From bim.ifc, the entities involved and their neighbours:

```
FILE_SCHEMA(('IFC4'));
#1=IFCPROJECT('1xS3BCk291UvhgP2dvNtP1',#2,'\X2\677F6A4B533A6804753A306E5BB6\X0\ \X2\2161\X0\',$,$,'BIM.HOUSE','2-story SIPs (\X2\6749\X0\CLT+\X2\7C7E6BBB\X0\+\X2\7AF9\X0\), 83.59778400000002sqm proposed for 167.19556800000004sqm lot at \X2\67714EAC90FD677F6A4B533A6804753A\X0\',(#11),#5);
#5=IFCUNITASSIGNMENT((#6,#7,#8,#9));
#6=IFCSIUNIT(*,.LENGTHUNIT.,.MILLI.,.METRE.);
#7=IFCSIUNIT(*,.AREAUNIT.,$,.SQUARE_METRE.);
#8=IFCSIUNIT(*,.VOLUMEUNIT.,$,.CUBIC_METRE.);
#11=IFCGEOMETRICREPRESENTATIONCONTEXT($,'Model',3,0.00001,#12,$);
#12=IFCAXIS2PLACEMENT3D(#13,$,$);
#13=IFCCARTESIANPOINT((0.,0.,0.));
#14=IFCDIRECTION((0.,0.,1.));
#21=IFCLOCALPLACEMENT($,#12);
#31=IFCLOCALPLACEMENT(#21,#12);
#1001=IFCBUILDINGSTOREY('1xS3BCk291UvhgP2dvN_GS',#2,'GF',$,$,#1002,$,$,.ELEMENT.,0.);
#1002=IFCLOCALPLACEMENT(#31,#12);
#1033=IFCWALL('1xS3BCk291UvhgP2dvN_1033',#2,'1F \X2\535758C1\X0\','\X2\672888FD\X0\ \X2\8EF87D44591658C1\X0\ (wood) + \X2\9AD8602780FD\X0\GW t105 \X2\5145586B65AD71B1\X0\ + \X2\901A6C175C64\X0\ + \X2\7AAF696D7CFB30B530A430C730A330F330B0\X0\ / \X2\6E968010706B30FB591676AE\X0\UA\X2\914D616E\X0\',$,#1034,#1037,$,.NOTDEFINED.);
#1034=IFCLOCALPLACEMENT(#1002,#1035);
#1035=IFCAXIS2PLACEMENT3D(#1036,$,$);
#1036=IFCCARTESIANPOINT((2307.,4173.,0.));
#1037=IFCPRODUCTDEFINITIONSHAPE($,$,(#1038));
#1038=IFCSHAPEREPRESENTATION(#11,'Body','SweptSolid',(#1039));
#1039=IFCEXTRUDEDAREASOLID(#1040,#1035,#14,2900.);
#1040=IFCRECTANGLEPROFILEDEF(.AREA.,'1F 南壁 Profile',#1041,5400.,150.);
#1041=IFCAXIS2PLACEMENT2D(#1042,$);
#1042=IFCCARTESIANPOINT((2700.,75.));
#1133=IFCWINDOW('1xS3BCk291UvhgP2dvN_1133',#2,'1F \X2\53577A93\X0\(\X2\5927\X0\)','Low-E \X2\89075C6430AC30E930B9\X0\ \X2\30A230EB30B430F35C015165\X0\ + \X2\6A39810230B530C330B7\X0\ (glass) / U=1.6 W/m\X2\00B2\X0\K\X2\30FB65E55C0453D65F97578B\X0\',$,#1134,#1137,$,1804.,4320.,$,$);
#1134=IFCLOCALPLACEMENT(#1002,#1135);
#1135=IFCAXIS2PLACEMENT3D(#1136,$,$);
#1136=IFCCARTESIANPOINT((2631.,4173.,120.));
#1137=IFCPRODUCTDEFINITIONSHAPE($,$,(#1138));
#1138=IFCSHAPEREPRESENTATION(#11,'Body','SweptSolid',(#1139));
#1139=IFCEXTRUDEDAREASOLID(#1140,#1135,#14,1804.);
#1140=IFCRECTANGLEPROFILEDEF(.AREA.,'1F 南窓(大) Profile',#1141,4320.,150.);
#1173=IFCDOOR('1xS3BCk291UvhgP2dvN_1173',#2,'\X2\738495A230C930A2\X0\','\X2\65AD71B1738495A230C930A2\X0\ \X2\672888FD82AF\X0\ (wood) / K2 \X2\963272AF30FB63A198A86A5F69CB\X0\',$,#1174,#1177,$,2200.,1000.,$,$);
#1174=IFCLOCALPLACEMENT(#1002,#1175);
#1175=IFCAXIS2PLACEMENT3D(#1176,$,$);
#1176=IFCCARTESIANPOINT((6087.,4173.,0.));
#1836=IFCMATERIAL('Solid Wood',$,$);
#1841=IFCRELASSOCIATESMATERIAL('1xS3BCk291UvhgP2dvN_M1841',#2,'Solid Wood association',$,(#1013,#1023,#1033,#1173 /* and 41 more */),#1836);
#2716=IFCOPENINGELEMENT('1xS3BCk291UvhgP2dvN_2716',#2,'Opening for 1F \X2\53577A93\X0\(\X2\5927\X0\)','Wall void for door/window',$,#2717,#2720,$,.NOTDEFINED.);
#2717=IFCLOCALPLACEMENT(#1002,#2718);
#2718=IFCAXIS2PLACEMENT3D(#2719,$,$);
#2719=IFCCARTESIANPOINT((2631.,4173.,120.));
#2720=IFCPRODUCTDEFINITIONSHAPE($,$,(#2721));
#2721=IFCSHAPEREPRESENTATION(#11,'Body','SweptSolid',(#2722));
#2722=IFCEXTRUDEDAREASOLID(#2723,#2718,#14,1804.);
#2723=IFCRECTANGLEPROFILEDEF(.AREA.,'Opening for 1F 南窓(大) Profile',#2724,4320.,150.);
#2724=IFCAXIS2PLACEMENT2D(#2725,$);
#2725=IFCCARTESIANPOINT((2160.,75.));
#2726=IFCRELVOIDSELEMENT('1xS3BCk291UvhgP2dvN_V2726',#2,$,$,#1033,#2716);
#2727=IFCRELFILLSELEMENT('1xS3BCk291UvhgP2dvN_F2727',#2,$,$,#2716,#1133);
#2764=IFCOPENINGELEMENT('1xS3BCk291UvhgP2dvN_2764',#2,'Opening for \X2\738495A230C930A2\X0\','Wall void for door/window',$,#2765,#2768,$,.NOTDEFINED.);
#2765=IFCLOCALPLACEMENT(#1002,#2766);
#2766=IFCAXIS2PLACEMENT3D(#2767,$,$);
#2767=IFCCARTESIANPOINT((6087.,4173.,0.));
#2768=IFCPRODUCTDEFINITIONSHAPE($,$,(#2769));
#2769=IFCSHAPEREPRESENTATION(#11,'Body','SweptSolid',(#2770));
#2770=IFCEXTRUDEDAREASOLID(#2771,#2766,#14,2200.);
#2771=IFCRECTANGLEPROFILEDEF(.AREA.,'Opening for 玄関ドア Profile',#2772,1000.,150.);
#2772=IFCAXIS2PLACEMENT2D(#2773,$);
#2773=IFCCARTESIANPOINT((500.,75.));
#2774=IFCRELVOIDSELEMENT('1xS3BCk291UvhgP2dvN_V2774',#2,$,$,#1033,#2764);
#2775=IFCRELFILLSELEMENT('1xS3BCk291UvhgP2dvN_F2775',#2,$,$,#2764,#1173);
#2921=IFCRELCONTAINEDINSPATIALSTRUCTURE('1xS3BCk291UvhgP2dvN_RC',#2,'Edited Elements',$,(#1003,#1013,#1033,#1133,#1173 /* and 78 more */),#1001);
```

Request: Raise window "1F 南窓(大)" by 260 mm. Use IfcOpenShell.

```python
import numpy as np
import ifcopenshell
import ifcopenshell.api.geometry
import ifcopenshell.util.placement
import ifcopenshell.util.unit

model = ifcopenshell.open("bim.ifc")
unit_scale = ifcopenshell.util.unit.calculate_unit_scale(model)

window = model.by_guid("1xS3BCk291UvhgP2dvN_1133")
opening = window.FillsVoids[0].RelatingOpeningElement
dz = 0.26 / unit_scale

shift = np.array([0.0, 0.0, dz])
# The window is not placed relative to its opening, so move both.
for product in (opening, window):
    matrix = ifcopenshell.util.placement.get_local_placement(product.ObjectPlacement)
    matrix[:3, 3] += shift
    ifcopenshell.api.geometry.edit_object_placement(model, product=product, matrix=matrix, is_si=False)

print(f"moved by {dz * unit_scale:+.3f} m")

model.write("bim_updated.ifc")
```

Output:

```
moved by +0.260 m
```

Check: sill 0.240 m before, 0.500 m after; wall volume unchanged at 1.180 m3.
